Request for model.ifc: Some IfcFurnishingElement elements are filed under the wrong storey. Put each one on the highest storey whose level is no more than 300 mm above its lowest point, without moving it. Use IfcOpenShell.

First a look at what the model holds.

```python
import ifcopenshell
import ifcopenshell.util.element
import ifcopenshell.util.placement

model = ifcopenshell.open("model.ifc")
print(model.schema)
for storey in model.by_type("IfcBuildingStorey"):
    level = ifcopenshell.util.placement.get_storey_elevation(storey)
    count = sum(e.is_a("IfcFurnishingElement") for e in ifcopenshell.util.element.get_contained(storey))
    print(storey.id(), storey.Name, round(level, 3), count, sep=" | ")
```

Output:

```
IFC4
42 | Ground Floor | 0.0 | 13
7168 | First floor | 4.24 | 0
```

```python
import ifcopenshell
import ifcopenshell.api.spatial
import ifcopenshell.geom
import ifcopenshell.util.element
import ifcopenshell.util.placement
import ifcopenshell.util.shape
import ifcopenshell.util.unit

model = ifcopenshell.open("model.ifc")
unit_scale = ifcopenshell.util.unit.calculate_unit_scale(model)
settings = ifcopenshell.geom.settings()

levels = sorted(
    ((ifcopenshell.util.placement.get_storey_elevation(s) * unit_scale, s) for s in model.by_type("IfcBuildingStorey")),
    key=lambda pair: pair[0],
)

for e in model.by_type("IfcFurnishingElement"):
    current = e.ContainedInStructure[0].RelatingStructure if e.ContainedInStructure else None
    if current is None or not current.is_a("IfcBuildingStorey"):
        continue
    shape = ifcopenshell.geom.create_shape(settings, e)
    bottom = ifcopenshell.util.shape.get_shape_bottom_elevation(shape, shape.geometry)
    below = [s for level, s in levels if level <= bottom + 0.3]
    storey = below[-1] if below else levels[0][1]
    if storey != current:
        # assign_container keeps the world position.
        ifcopenshell.api.spatial.assign_container(model, products=[e], relating_structure=storey)
        print(e.id(), current.Name, "->", storey.Name)

model.write("model_updated.ifc")
```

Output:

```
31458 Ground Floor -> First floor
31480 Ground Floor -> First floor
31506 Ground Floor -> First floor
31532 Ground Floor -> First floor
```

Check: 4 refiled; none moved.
